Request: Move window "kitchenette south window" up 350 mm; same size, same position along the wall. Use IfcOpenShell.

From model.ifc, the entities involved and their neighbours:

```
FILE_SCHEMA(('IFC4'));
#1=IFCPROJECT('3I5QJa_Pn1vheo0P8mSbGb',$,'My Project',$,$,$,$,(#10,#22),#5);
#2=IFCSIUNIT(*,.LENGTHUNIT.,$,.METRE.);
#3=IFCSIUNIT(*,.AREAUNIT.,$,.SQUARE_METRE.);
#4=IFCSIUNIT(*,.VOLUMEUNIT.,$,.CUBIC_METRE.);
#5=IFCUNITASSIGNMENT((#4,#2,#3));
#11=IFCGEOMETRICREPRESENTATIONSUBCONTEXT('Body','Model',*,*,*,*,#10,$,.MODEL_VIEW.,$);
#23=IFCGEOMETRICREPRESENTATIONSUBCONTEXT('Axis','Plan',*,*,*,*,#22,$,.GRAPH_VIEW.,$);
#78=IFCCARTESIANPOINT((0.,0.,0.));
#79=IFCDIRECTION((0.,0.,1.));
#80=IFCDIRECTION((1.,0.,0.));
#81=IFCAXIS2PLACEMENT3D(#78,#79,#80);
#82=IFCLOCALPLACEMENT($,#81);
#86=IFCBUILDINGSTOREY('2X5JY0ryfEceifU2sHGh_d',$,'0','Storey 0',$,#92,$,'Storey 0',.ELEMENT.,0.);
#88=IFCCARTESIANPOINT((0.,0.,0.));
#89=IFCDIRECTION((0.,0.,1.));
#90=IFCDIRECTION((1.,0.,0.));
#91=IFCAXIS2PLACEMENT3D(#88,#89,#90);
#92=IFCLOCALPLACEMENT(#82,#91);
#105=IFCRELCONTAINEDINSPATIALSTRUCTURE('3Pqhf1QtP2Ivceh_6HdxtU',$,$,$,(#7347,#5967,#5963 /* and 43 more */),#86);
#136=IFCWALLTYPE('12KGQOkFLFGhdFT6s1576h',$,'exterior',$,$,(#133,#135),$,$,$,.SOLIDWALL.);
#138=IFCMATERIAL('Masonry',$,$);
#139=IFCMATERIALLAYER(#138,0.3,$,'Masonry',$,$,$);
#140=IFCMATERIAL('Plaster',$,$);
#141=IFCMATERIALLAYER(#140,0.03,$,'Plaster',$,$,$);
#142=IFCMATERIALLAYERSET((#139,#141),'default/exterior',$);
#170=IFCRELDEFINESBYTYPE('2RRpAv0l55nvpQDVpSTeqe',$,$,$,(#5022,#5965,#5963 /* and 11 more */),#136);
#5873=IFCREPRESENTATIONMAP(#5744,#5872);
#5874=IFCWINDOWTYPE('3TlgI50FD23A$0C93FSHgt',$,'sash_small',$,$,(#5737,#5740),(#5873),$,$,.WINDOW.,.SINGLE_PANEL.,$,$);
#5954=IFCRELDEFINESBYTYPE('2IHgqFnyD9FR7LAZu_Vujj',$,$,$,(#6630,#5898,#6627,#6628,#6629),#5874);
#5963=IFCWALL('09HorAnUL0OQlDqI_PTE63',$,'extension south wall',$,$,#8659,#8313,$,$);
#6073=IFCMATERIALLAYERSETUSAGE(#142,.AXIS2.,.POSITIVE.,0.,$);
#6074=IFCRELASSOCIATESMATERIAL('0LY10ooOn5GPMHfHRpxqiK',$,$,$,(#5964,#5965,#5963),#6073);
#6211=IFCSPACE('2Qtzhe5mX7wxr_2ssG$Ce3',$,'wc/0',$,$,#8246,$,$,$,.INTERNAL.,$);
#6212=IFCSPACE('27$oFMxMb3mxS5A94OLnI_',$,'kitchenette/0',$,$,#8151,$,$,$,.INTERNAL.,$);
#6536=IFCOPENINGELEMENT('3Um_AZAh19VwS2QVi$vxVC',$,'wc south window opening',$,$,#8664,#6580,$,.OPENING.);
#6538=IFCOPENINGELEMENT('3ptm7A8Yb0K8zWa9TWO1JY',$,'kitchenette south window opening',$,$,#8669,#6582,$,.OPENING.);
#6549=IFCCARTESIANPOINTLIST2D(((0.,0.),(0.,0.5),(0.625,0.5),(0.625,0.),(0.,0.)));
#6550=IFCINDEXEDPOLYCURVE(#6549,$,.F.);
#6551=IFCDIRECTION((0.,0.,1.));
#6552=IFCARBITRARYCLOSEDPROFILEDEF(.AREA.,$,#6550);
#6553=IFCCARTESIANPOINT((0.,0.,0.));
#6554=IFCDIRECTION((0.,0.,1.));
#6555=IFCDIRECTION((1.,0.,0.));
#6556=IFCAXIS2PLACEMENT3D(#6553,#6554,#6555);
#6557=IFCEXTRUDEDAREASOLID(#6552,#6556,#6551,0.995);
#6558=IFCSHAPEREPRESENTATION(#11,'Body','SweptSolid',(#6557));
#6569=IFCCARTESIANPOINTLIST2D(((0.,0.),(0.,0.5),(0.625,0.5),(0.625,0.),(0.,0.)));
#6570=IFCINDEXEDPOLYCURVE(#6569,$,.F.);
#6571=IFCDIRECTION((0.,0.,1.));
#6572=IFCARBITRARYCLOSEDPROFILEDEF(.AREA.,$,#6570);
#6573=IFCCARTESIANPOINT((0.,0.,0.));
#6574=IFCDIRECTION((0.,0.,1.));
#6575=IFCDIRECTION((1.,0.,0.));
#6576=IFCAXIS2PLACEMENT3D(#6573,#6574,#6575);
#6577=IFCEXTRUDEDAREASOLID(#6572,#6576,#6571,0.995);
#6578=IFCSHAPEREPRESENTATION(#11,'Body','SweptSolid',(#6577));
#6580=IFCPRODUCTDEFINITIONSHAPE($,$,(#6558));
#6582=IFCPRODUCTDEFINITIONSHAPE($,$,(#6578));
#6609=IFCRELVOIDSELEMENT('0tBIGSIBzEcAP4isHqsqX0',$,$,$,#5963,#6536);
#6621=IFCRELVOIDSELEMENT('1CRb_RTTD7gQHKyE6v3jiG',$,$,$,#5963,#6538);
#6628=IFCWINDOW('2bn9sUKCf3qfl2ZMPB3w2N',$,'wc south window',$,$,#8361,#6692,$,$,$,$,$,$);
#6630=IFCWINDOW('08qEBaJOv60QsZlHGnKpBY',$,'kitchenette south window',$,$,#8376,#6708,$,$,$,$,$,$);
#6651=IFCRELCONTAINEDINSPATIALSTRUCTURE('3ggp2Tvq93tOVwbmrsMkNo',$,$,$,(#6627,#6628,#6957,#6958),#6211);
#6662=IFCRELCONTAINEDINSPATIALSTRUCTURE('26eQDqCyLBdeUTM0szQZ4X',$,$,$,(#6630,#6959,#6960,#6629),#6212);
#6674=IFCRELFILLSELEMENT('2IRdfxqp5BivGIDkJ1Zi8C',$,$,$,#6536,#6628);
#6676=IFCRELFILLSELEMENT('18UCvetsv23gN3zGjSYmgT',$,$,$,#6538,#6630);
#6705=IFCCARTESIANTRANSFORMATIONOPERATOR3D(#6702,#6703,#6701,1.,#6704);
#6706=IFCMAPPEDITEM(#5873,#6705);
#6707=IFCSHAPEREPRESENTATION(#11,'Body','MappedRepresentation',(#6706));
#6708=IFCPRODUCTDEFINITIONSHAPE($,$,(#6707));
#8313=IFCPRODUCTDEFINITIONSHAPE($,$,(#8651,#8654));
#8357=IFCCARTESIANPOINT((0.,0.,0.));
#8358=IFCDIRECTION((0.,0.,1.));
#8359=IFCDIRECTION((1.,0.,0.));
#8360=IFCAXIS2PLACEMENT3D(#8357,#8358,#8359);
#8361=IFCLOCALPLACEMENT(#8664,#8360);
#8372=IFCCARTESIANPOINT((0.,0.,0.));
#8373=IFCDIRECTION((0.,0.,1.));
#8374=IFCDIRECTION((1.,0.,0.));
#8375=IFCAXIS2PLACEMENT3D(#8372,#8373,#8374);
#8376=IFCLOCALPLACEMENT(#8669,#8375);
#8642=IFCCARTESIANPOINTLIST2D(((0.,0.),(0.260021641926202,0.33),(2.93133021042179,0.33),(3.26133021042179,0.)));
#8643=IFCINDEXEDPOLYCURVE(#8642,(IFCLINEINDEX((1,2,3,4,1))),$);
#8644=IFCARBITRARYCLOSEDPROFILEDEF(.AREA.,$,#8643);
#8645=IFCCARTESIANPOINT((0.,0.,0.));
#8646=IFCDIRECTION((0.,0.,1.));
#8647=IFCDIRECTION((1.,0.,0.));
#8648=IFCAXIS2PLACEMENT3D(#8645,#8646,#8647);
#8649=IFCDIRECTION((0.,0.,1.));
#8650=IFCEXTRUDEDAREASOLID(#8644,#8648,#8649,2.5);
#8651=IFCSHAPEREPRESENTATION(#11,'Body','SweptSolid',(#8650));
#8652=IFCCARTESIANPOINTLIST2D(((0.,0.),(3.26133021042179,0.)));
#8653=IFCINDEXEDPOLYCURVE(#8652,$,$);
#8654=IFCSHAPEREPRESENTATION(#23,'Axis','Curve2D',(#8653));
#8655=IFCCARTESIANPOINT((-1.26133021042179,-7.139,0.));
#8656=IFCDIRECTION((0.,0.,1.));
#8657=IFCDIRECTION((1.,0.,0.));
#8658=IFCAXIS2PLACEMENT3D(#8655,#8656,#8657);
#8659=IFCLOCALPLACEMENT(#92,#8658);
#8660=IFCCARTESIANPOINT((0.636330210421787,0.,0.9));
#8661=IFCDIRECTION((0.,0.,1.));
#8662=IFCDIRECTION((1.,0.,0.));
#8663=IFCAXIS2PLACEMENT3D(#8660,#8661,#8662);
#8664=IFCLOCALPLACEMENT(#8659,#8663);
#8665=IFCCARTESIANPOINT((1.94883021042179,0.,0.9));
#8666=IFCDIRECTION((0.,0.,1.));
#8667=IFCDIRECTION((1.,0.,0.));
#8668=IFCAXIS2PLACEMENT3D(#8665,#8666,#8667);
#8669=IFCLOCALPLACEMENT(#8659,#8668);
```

```python
import numpy as np
import ifcopenshell
import ifcopenshell.api.geometry
import ifcopenshell.util.placement
import ifcopenshell.util.unit

model = ifcopenshell.open("model.ifc")
unit_scale = ifcopenshell.util.unit.calculate_unit_scale(model)

window = model.by_id(6630)
opening = window.FillsVoids[0].RelatingOpeningElement
dz = 0.35 / unit_scale

shift = np.array([0.0, 0.0, dz])
# The window is placed relative to its opening, so it follows when the opening moves.
matrix = ifcopenshell.util.placement.get_local_placement(opening.ObjectPlacement)
matrix[:3, 3] += shift
ifcopenshell.api.geometry.edit_object_placement(
    model, product=opening, matrix=matrix, is_si=False, should_transform_children=True
)

print(f"moved by {dz * unit_scale:+.3f} m")

model.write("model-out.ifc")
```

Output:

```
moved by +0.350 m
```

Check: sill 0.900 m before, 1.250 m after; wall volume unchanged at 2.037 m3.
